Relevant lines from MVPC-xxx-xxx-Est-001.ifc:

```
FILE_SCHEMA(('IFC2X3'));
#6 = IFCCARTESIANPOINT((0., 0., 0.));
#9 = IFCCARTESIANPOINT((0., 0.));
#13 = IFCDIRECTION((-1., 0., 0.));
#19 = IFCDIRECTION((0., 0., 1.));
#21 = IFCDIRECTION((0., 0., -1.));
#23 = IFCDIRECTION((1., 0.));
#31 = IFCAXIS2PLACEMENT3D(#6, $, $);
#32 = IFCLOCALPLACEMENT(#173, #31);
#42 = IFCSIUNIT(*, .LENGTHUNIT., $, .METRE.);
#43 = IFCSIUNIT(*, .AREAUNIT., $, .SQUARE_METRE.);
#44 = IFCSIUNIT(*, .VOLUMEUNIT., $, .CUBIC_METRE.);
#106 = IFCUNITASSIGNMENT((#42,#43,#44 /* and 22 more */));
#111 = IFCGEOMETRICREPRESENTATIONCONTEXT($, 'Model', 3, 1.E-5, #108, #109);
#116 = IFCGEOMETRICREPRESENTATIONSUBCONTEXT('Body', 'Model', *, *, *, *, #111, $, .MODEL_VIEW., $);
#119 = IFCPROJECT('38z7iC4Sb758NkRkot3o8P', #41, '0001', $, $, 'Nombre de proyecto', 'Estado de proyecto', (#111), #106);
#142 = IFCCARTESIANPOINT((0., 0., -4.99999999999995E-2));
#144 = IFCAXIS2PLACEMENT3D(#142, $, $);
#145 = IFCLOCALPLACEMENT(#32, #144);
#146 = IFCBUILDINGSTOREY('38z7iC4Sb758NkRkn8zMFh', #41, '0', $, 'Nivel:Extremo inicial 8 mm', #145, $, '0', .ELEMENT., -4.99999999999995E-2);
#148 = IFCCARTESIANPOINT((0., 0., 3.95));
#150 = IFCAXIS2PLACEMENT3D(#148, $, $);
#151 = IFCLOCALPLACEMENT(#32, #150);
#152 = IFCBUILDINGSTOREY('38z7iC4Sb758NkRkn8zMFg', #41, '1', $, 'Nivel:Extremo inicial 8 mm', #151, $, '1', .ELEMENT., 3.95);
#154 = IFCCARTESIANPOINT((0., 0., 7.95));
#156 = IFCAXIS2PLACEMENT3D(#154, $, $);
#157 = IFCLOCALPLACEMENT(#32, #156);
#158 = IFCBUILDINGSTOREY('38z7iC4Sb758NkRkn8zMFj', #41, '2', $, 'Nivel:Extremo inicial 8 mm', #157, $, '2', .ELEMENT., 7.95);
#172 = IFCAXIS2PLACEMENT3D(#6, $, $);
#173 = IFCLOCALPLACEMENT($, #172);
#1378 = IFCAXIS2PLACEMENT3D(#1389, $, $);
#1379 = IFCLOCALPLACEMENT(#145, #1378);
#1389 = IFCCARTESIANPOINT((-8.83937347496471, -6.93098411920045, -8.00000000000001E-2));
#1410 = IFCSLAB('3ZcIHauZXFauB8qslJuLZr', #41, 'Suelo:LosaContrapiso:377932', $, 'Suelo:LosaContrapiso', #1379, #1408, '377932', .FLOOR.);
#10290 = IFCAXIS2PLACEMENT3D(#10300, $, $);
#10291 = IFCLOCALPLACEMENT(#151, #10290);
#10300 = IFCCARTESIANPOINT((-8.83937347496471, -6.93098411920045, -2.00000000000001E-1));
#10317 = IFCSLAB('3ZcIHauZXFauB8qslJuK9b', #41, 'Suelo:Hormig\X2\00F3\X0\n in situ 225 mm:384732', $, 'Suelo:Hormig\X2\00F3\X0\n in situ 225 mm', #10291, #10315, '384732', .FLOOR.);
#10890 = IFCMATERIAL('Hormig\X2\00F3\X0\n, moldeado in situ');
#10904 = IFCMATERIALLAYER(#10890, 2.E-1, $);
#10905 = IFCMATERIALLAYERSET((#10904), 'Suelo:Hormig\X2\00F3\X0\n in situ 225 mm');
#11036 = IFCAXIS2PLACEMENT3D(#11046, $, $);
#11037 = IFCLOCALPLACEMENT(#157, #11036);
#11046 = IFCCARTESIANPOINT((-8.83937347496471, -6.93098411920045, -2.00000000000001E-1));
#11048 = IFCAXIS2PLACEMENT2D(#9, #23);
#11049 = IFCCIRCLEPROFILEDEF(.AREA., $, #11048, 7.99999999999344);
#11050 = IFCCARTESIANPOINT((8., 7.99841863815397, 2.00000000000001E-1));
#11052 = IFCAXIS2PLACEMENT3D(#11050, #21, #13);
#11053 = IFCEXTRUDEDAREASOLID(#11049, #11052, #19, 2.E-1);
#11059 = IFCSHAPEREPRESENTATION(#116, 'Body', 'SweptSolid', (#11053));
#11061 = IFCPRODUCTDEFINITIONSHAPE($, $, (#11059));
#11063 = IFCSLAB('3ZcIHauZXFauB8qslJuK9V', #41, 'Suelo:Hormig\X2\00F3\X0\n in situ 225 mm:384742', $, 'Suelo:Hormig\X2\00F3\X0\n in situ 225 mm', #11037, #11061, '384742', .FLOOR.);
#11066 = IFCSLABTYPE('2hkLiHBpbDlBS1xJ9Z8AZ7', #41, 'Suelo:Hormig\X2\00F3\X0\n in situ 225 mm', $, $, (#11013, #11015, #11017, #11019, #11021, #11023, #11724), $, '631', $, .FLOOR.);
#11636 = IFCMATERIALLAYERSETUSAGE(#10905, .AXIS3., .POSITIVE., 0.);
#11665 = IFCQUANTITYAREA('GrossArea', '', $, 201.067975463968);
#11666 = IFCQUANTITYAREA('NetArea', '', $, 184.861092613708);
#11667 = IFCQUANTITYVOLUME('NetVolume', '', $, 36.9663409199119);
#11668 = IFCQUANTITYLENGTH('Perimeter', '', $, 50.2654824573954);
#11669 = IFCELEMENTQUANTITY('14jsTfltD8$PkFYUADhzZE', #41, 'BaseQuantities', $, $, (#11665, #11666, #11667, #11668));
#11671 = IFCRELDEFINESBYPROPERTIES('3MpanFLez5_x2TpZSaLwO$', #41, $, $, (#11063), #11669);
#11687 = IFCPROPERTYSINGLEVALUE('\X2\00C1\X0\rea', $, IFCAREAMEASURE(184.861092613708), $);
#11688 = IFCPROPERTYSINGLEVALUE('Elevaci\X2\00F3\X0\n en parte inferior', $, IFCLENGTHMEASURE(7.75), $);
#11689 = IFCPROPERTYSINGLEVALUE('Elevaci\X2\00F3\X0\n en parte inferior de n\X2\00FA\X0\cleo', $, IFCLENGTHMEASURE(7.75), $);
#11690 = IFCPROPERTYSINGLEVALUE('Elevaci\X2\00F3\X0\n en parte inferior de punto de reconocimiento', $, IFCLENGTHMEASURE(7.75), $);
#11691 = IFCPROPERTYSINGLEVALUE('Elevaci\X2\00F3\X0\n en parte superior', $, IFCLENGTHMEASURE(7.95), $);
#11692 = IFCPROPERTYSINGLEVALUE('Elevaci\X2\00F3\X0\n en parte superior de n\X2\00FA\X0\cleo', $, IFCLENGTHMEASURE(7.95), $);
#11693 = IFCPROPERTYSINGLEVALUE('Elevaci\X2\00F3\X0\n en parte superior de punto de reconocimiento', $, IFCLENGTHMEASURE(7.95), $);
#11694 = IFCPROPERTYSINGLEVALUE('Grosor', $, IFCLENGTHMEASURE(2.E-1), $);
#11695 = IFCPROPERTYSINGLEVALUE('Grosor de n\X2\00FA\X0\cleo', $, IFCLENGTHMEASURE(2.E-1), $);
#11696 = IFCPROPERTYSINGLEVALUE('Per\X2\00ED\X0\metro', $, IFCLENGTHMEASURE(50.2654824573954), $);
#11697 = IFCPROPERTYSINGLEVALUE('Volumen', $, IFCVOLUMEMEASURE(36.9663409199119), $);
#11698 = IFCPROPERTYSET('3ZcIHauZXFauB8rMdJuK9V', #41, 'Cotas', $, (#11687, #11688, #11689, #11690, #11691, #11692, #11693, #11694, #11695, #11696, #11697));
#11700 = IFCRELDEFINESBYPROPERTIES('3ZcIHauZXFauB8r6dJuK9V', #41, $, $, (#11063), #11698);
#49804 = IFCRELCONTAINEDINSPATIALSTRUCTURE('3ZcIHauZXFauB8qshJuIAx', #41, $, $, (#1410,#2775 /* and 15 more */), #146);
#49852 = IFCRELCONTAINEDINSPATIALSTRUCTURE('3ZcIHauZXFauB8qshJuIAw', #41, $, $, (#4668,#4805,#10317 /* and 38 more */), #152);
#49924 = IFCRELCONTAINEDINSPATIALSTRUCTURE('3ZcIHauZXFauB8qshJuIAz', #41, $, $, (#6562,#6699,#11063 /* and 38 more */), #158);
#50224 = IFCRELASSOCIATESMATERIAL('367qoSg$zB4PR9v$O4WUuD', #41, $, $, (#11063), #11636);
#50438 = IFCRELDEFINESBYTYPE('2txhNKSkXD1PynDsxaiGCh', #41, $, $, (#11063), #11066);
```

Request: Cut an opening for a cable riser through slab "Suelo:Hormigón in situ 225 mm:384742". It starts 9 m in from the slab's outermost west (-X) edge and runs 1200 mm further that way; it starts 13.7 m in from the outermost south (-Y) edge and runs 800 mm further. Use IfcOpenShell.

```python
import numpy as np
import ifcopenshell
import ifcopenshell.api.feature
import ifcopenshell.api.geometry
import ifcopenshell.api.pset
import ifcopenshell.api.root
import ifcopenshell.geom
import ifcopenshell.util.element
import ifcopenshell.util.placement
import ifcopenshell.util.representation
import ifcopenshell.util.shape
import ifcopenshell.util.unit

model = ifcopenshell.open("MVPC-xxx-xxx-Est-001.ifc")
unit_scale = ifcopenshell.util.unit.calculate_unit_scale(model)
area_scale = ifcopenshell.util.unit.calculate_unit_scale(model, "AREAUNIT")
volume_scale = ifcopenshell.util.unit.calculate_unit_scale(model, "VOLUMEUNIT")
settings = ifcopenshell.geom.settings()


def volume(element):
    """Net volume in cubic metres, openings subtracted."""
    shape = ifcopenshell.geom.create_shape(settings, element)
    return ifcopenshell.util.shape.get_volume(shape.geometry)


slab = model.by_guid("3ZcIHauZXFauB8qslJuK9V")
before = volume(slab)

# Extent in the slab's own axes, in metres. The edges named are its -X and -Y sides.
slab_shape = ifcopenshell.geom.create_shape(settings, slab)
vertices = ifcopenshell.util.shape.get_vertices(slab_shape.geometry)
x_min, y_min, bottom = vertices.min(axis=0)
top = vertices[:, 2].max()

opening = ifcopenshell.api.root.create_entity(model, ifc_class="IfcOpeningElement", name="Cable riser opening")
context = ifcopenshell.util.representation.get_context(model, "Model", "Body", "MODEL_VIEW")
width, depth = 1.2, 0.8
outline = [(0.0, 0.0), (width, 0.0), (width, depth), (0.0, depth), (0.0, 0.0)]
# Overshoot both faces by 50 mm so the cut is clean.
shape = ifcopenshell.api.geometry.add_slab_representation(
    model, context=context, depth=top - bottom + 0.1, polyline=outline
)
ifcopenshell.api.geometry.assign_representation(model, product=opening, representation=shape)

matrix = ifcopenshell.util.placement.get_local_placement(slab.ObjectPlacement)
matrix[:, 3] = matrix @ np.append(np.array([x_min + 9, y_min + 13.7, bottom - 0.05]) / unit_scale, 1.0)
ifcopenshell.api.geometry.edit_object_placement(model, product=opening, matrix=matrix, is_si=False)
ifcopenshell.api.feature.add_feature(model, feature=opening, element=slab)

after = volume(slab)

# Update the slab's stored quantities.
qto = model.by_id(ifcopenshell.util.element.get_pset(slab, "BaseQuantities", should_inherit=False)["id"])
ifcopenshell.api.pset.edit_qto(model, qto=qto, properties={
    "NetArea": after / (top - bottom) / area_scale,
    "NetVolume": after / volume_scale,
})
pset = model.by_id(ifcopenshell.util.element.get_pset(slab, "Cotas", should_inherit=False)["id"])
ifcopenshell.api.pset.edit_pset(model, pset=pset, properties={
    "Área": model.create_entity("IfcAreaMeasure", after / (top - bottom) / area_scale),
    "Volumen": model.create_entity("IfcVolumeMeasure", after / volume_scale),
})

print(f"slab volume {before:.3f} -> {after:.3f} m3")

model.write("MVPC-xxx-xxx-Est-001_edited.ifc")
```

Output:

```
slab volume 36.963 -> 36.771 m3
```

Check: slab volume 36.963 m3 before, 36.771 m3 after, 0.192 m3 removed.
